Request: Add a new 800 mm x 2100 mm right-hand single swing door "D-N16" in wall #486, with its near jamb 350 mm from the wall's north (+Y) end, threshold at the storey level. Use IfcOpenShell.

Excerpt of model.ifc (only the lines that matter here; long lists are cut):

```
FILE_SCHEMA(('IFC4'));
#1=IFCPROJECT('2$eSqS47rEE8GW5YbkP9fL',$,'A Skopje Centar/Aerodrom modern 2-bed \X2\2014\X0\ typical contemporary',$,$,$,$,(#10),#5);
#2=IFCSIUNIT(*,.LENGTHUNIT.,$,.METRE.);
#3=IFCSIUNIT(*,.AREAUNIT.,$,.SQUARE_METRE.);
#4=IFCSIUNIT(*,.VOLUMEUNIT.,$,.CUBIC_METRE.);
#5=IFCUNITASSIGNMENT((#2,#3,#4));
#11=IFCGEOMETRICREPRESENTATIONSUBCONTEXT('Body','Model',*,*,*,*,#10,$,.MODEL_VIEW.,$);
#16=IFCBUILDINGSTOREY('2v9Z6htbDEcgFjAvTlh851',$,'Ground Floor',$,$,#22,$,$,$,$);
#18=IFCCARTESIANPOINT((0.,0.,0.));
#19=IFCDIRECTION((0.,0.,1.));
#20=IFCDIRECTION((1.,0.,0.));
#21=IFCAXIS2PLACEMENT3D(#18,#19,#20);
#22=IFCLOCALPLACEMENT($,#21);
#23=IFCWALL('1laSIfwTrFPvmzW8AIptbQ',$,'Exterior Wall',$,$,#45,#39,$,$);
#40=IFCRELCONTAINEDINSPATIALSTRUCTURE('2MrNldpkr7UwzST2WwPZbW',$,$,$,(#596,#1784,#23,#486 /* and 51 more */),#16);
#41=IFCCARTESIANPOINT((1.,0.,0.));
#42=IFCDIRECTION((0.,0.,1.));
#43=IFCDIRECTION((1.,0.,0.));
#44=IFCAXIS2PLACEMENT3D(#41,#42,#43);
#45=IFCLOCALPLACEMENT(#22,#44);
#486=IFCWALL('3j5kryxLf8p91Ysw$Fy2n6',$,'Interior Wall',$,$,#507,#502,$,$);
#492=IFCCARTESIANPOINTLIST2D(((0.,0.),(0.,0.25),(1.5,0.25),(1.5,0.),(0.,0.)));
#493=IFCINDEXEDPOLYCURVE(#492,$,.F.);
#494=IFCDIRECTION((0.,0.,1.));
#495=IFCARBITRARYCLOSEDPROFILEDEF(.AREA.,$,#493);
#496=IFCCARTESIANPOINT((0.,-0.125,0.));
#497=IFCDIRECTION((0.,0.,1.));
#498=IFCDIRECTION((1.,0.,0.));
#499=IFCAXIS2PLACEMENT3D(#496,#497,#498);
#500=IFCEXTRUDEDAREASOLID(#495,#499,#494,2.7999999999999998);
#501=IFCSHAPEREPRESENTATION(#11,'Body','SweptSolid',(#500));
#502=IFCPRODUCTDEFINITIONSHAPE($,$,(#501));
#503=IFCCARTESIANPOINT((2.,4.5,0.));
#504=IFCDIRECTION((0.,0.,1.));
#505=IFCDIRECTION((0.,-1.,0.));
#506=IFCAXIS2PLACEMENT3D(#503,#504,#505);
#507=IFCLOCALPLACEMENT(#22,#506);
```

```python
import numpy as np
import ifcopenshell
import ifcopenshell.api.feature
import ifcopenshell.api.geometry
import ifcopenshell.api.root
import ifcopenshell.api.spatial
import ifcopenshell.geom
import ifcopenshell.util.element
import ifcopenshell.util.placement
import ifcopenshell.util.representation
import ifcopenshell.util.shape
import ifcopenshell.util.unit

model = ifcopenshell.open("model.ifc")
unit_scale = ifcopenshell.util.unit.calculate_unit_scale(model)
settings = ifcopenshell.geom.settings()


def volume(element):
    """Net volume in cubic metres, openings subtracted."""
    shape = ifcopenshell.geom.create_shape(settings, element)
    return ifcopenshell.util.shape.get_volume(shape.geometry)


wall = model.by_guid("3j5kryxLf8p91Ysw$Fy2n6")
storey = ifcopenshell.util.element.get_container(wall, ifc_class="IfcBuildingStorey")
context = ifcopenshell.util.representation.get_context(model, "Model", "Body", "MODEL_VIEW")
before = volume(wall)

width, height, from_end, sill = 0.8, 2.1, 0.35, 0.0  # metres

# The wall runs along its own X axis, and the end named is its -X end.
wall_shape = ifcopenshell.geom.create_shape(settings, wall)
x, y, z = ifcopenshell.util.shape.get_vertices(wall_shape.geometry).T
start = x.min() + from_end
face, thickness = float(y.min()), float(y.max() - y.min())
wall_matrix = ifcopenshell.util.placement.get_local_placement(wall.ObjectPlacement)
level = ifcopenshell.util.placement.get_local_placement(storey.ObjectPlacement)[2, 3]


def in_wall(x, y):
    """Placement at x, y metres in the wall's axes, at sill height."""
    matrix = wall_matrix.copy()
    matrix[:, 3] = wall_matrix @ np.array([x / unit_scale, y / unit_scale, 0.0, 1.0])
    matrix[2, 3] = level + sill / unit_scale
    return matrix


# Opening: a box that overshoots both wall faces by 50 mm.
opening = ifcopenshell.api.root.create_entity(model, ifc_class="IfcOpeningElement", predefined_type="OPENING")
box = ifcopenshell.api.geometry.add_wall_representation(
    model, context=context, length=width, height=height, thickness=thickness + 0.1
)
ifcopenshell.api.geometry.assign_representation(model, product=opening, representation=box)
ifcopenshell.api.geometry.edit_object_placement(model, product=opening, matrix=in_wall(start, face - 0.05), is_si=False)
ifcopenshell.api.feature.add_feature(model, feature=opening, element=wall)

door = ifcopenshell.api.root.create_entity(model, ifc_class="IfcDoor", name="D-N16", predefined_type="DOOR")
door.OverallWidth, door.OverallHeight = width / unit_scale, height / unit_scale
door.OperationType = "SINGLE_SWING_RIGHT"
body = ifcopenshell.api.geometry.add_door_representation(
    model,
    context=context,
    overall_width=door.OverallWidth,
    overall_height=door.OverallHeight,
    operation_type="SINGLE_SWING_RIGHT",
    lining_properties={"LiningDepth": thickness / unit_scale, "ThresholdDepth": thickness / unit_scale},
)
ifcopenshell.api.geometry.assign_representation(model, product=door, representation=body)
ifcopenshell.api.spatial.assign_container(model, products=[door], relating_structure=storey)
ifcopenshell.api.feature.add_filling(model, opening=opening, element=door)

# The lining spans the wall, so the door starts at the wall face.
ifcopenshell.api.geometry.edit_object_placement(model, product=door, matrix=in_wall(start, face), is_si=False)

after = volume(wall)

print(f"wall volume {before:.3f} -> {after:.3f} m3")

model.write("model_edited.ifc")
```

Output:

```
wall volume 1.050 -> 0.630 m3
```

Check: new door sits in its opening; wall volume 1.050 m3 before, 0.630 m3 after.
